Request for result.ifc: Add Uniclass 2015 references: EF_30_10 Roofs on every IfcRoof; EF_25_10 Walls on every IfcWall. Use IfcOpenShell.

First a look at what the model holds.

```python
import ifcopenshell

model = ifcopenshell.open("result.ifc")
print(model.schema)
print("classifications:", [c.Name for c in model.by_type("IfcClassification")])
for ifc_class in ("IfcDoor", "IfcRoof", "IfcStair", "IfcWall", "IfcWindow"):
    print(ifc_class, len(model.by_type(ifc_class)))
```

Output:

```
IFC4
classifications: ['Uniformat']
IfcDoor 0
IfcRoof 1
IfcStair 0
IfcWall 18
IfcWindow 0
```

```python
import ifcopenshell
import ifcopenshell.api.classification

model = ifcopenshell.open("result.ifc")

system = ifcopenshell.api.classification.add_classification(model, classification="Uniclass 2015")

codes = {
    "IfcRoof": ("EF_30_10", "Roofs"),
    "IfcWall": ("EF_25_10", "Walls"),
}
for ifc_class, (code, name) in codes.items():
    products = model.by_type(ifc_class)
    ifcopenshell.api.classification.add_reference(
        model, products=products, classification=system, identification=code, name=name
    )
    print(code, len(products))

model.write("result-out.ifc")
```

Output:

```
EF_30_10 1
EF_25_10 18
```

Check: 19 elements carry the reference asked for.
